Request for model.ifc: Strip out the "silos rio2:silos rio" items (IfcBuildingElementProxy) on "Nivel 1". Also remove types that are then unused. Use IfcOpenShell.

First a look at what the model holds.

```python
import ifcopenshell
import ifcopenshell.util.element

model = ifcopenshell.open("model.ifc")
print(model.schema)
storey = next(s for s in model.by_type("IfcBuildingStorey") if s.Name == "Nivel 1")
proxies = [e for e in ifcopenshell.util.element.get_decomposition(storey) if e.is_a("IfcBuildingElementProxy")]
seen = {}
for e in proxies:
    element_type = ifcopenshell.util.element.get_type(e)
    name = element_type.Name if element_type not in (None, e) else None
    seen[name] = seen.get(name, 0) + 1
for name, count in sorted(seen.items(), key=str):
    print(count, "x", name)
```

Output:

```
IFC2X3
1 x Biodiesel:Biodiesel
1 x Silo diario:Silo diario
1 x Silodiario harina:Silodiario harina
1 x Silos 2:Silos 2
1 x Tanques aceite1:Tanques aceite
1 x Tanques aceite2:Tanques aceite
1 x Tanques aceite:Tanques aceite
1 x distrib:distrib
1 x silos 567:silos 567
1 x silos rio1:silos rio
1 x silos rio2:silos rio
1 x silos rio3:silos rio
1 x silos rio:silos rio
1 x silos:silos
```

```python
import ifcopenshell
import ifcopenshell.api.root
import ifcopenshell.util.element

model = ifcopenshell.open("model.ifc")

storey = next(s for s in model.by_type("IfcBuildingStorey") if s.Name == "Nivel 1")
proxies = [e for e in ifcopenshell.util.element.get_decomposition(storey) if e.is_a("IfcBuildingElementProxy")]
targets = [e for e in proxies if (t := ifcopenshell.util.element.get_type(e)) not in (None, e) and t.Name == "silos rio2:silos rio"]
types = {ifcopenshell.util.element.get_type(e) for e in targets} - {None, *targets}

for e in targets:
    ifcopenshell.api.root.remove_product(model, product=e)
print(len(targets), "removed")

unused = [t for t in types if not ifcopenshell.util.element.get_types(t)]
for t in unused:
    ifcopenshell.api.root.remove_product(model, product=t)
print(len(unused), "unused types removed")

model.write("model_edited.ifc")
```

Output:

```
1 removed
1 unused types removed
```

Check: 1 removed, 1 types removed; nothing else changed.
